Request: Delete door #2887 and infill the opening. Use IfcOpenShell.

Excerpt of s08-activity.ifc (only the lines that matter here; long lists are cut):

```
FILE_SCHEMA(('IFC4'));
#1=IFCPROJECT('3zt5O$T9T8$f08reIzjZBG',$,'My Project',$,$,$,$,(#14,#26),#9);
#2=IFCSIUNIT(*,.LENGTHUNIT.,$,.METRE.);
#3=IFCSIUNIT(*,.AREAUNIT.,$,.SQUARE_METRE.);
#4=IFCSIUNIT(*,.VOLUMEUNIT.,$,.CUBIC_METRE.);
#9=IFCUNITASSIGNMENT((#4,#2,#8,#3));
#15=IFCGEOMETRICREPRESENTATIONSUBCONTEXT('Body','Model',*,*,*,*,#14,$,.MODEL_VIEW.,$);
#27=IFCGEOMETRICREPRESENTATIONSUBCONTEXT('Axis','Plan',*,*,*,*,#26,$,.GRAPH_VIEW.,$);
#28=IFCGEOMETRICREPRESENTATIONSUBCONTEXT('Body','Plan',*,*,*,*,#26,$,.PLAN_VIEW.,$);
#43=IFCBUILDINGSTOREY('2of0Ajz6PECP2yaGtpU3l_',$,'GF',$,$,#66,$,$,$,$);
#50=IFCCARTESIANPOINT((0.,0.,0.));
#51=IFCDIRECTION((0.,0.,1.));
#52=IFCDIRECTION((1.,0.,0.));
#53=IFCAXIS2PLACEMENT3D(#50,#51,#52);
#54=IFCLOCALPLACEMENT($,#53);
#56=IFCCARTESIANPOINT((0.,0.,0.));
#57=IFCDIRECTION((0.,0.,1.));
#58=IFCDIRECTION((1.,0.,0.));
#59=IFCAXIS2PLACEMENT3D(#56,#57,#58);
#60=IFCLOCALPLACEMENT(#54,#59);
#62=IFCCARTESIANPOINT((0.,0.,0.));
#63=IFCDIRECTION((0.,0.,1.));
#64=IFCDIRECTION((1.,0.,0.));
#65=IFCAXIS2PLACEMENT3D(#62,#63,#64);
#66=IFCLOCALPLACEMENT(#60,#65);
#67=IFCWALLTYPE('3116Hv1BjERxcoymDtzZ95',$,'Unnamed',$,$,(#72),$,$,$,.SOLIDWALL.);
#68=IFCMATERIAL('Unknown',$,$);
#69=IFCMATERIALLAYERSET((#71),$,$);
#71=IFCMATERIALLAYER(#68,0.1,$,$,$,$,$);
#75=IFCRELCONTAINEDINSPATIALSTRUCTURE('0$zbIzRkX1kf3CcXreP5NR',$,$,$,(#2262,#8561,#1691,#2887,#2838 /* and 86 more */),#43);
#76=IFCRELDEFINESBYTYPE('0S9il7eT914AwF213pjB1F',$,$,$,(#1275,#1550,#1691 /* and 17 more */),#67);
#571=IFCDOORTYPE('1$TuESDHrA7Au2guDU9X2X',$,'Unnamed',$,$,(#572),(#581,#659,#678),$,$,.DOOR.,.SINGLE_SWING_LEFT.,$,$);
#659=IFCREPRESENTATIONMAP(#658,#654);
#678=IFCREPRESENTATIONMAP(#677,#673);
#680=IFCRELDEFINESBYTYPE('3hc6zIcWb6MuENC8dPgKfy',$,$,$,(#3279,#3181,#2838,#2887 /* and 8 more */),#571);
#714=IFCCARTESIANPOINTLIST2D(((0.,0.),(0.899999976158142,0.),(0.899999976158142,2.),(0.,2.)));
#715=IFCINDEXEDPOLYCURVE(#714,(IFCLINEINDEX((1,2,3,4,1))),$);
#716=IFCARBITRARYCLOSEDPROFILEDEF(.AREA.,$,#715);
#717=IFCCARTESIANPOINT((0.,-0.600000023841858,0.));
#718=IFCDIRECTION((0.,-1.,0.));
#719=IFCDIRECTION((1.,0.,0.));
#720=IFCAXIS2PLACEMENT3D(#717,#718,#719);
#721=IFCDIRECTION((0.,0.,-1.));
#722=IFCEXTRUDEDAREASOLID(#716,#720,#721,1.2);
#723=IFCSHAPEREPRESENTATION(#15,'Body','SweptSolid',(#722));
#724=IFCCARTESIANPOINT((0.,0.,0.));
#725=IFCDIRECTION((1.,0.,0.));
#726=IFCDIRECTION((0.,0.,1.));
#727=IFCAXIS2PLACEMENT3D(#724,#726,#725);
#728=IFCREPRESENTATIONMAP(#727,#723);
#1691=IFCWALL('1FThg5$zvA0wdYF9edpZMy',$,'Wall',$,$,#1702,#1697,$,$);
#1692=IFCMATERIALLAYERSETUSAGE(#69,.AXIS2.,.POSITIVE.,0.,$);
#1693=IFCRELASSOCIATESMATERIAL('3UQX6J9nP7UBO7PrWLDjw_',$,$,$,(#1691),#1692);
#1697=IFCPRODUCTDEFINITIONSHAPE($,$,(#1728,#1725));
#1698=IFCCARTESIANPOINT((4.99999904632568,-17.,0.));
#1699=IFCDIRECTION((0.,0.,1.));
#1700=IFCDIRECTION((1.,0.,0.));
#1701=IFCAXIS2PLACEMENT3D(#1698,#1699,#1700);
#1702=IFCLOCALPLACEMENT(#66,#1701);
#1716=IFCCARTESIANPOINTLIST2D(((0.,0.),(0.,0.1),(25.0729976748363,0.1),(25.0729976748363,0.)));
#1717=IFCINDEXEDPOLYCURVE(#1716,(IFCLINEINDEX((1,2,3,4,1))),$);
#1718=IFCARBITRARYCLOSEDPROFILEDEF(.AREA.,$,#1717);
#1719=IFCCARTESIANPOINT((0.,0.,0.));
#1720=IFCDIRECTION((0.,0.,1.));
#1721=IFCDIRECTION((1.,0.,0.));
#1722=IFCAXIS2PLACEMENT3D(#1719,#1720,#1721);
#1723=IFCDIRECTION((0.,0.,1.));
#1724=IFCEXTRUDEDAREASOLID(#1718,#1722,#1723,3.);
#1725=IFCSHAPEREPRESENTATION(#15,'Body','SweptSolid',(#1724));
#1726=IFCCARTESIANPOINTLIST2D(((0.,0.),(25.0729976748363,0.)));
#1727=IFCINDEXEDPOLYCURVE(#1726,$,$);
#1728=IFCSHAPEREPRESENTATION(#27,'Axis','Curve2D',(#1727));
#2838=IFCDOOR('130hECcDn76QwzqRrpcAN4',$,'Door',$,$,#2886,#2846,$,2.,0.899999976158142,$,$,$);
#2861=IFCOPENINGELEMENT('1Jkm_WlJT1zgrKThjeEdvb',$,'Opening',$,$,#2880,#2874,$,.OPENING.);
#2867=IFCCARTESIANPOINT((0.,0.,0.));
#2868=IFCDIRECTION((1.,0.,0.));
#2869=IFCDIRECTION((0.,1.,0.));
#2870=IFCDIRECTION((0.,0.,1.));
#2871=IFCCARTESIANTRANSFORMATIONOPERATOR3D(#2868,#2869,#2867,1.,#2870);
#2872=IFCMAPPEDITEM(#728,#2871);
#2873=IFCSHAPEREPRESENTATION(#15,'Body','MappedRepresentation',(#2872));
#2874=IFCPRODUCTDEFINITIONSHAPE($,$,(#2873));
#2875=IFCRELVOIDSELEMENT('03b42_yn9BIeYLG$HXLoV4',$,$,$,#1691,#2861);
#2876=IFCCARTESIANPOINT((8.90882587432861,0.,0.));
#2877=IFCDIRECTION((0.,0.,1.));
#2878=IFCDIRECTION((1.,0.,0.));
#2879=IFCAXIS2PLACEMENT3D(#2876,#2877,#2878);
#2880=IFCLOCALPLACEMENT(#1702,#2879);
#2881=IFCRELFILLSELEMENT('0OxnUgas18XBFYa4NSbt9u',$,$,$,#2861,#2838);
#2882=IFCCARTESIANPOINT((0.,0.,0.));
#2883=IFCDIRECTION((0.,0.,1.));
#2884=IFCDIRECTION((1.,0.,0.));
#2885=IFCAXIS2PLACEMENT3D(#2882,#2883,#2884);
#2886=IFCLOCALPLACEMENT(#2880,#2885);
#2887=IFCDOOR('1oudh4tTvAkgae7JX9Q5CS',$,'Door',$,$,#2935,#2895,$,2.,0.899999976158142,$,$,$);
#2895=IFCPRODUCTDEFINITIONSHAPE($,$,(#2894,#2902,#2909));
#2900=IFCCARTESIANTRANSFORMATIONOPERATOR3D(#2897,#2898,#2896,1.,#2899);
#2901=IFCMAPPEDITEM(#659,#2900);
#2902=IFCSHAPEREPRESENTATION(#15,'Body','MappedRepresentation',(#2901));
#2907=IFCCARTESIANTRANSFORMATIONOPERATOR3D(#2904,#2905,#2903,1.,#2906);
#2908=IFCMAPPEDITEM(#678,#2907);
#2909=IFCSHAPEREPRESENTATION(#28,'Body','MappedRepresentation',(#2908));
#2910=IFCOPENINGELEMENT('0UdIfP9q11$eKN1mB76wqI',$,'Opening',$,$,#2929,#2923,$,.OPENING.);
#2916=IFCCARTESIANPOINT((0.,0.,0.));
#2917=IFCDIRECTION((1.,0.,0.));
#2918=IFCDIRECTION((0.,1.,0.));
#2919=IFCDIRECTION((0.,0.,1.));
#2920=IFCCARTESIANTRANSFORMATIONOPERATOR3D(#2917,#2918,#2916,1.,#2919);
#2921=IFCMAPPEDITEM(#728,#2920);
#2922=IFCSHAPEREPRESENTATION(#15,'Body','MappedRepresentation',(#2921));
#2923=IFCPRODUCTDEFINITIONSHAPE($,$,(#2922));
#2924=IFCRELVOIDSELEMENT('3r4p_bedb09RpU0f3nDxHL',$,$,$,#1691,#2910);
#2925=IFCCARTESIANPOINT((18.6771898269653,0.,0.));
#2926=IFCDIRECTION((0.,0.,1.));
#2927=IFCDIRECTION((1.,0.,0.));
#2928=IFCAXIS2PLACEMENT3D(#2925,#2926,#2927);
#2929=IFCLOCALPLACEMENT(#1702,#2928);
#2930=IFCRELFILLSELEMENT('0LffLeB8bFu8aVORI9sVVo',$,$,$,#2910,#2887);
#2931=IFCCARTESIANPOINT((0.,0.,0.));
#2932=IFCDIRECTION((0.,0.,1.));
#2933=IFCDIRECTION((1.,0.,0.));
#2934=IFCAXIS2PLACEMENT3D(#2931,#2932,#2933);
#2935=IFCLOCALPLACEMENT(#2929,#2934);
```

```python
import ifcopenshell
import ifcopenshell.api.feature
import ifcopenshell.api.root
import ifcopenshell.geom
import ifcopenshell.util.shape

model = ifcopenshell.open("s08-activity.ifc")
settings = ifcopenshell.geom.settings()


def volume(element):
    """Net volume in cubic metres, openings subtracted."""
    shape = ifcopenshell.geom.create_shape(settings, element)
    return ifcopenshell.util.shape.get_volume(shape.geometry)


door = model.by_id(2887)
opening = door.FillsVoids[0].RelatingOpeningElement
wall = opening.VoidsElements[0].RelatingBuildingElement
before = volume(wall)

ifcopenshell.api.root.remove_product(model, product=door)
ifcopenshell.api.feature.remove_feature(model, feature=opening)

after = volume(wall)

print(f"wall volume {before:.3f} -> {after:.3f} m3")

model.write("s08-activity_updated.ifc")
```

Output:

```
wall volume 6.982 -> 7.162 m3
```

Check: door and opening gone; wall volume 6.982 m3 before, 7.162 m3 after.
